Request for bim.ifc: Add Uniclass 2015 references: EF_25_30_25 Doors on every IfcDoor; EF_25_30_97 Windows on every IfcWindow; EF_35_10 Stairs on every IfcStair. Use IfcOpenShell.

First a look at what the model holds.

```python
import ifcopenshell

model = ifcopenshell.open("bim.ifc")
print(model.schema)
print("classifications:", [c.Name for c in model.by_type("IfcClassification")])
for ifc_class in ("IfcDoor", "IfcRoof", "IfcStair", "IfcWall", "IfcWindow"):
    print(ifc_class, len(model.by_type(ifc_class)))
```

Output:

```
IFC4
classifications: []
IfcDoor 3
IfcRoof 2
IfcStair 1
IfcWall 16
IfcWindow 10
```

```python
import ifcopenshell
import ifcopenshell.api.classification

model = ifcopenshell.open("bim.ifc")

system = ifcopenshell.api.classification.add_classification(model, classification="Uniclass 2015")

codes = {
    "IfcDoor": ("EF_25_30_25", "Doors"),
    "IfcWindow": ("EF_25_30_97", "Windows"),
    "IfcStair": ("EF_35_10", "Stairs"),
}
for ifc_class, (code, name) in codes.items():
    products = model.by_type(ifc_class)
    ifcopenshell.api.classification.add_reference(
        model, products=products, classification=system, identification=code, name=name
    )
    print(code, len(products))

model.write("bim_updated.ifc")
```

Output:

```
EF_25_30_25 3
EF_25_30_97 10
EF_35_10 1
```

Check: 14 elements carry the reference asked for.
